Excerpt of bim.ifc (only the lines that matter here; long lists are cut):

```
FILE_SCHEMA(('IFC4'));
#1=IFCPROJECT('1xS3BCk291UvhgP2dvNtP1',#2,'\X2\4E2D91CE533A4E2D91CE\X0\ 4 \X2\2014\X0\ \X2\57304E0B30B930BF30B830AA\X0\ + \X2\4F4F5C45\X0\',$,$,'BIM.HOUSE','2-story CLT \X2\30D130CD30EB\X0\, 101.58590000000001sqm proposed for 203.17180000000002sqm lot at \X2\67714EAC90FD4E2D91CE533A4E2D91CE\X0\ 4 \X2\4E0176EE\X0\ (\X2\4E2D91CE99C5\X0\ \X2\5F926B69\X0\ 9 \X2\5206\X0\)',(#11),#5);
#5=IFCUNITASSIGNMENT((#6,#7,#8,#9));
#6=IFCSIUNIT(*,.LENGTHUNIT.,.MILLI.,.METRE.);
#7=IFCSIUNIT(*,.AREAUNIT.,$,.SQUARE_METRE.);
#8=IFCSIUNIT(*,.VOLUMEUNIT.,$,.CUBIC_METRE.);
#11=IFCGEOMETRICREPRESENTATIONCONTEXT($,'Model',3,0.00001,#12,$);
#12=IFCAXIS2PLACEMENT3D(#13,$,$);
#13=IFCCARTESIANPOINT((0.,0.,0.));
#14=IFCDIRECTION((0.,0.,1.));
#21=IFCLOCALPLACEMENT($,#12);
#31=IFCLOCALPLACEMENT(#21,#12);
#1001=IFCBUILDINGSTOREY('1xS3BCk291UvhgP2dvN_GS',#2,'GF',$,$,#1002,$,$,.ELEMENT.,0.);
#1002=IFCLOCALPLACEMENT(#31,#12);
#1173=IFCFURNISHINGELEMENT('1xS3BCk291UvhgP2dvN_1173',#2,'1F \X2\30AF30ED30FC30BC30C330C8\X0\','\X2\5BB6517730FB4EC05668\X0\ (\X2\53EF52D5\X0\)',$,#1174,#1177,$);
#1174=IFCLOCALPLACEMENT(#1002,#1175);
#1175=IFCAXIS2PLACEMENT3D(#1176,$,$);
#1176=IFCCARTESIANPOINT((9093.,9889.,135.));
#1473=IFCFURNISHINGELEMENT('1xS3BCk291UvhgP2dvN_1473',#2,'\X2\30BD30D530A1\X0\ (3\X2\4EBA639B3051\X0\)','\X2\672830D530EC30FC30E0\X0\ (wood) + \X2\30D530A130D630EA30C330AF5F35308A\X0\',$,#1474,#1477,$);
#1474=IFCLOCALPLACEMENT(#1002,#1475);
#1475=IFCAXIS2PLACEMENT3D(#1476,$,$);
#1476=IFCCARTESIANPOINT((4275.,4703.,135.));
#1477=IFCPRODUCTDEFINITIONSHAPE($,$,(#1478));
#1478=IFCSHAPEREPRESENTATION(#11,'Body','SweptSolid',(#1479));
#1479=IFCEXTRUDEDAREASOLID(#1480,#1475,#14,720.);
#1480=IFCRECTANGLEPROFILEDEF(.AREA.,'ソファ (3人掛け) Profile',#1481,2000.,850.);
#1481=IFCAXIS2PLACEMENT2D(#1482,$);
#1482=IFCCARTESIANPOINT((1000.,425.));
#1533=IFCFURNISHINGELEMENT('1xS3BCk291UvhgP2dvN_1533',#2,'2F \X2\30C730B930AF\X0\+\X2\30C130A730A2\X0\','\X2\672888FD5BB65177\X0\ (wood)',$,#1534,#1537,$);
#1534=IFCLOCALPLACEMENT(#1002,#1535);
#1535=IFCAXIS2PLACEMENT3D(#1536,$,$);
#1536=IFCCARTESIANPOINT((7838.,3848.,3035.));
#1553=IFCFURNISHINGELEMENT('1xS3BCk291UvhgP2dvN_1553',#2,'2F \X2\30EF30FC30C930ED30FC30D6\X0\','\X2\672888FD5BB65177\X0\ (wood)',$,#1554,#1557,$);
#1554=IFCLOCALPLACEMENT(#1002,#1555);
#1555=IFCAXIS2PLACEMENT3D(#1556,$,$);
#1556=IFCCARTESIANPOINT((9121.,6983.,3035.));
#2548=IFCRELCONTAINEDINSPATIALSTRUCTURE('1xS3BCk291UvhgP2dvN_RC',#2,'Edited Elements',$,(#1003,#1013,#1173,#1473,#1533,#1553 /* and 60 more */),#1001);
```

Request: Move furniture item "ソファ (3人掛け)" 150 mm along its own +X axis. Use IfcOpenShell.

```python
import ifcopenshell
import ifcopenshell.api.geometry
import ifcopenshell.util.placement

model = ifcopenshell.open("bim.ifc")

item = model.by_guid("1xS3BCk291UvhgP2dvN_1473")
matrix = ifcopenshell.util.placement.get_local_placement(item.ObjectPlacement)
matrix[:3, 3] += matrix[:3, 0] * 150.0
ifcopenshell.api.geometry.edit_object_placement(model, product=item, matrix=matrix, is_si=False)

print(ifcopenshell.util.placement.get_local_placement(item.ObjectPlacement).round(3) + 0.0)

model.write("bim_edited.ifc")
```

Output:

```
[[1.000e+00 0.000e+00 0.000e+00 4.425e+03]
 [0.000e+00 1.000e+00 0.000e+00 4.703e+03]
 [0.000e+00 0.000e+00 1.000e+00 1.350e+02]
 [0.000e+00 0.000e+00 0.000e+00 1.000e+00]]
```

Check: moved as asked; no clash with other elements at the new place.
